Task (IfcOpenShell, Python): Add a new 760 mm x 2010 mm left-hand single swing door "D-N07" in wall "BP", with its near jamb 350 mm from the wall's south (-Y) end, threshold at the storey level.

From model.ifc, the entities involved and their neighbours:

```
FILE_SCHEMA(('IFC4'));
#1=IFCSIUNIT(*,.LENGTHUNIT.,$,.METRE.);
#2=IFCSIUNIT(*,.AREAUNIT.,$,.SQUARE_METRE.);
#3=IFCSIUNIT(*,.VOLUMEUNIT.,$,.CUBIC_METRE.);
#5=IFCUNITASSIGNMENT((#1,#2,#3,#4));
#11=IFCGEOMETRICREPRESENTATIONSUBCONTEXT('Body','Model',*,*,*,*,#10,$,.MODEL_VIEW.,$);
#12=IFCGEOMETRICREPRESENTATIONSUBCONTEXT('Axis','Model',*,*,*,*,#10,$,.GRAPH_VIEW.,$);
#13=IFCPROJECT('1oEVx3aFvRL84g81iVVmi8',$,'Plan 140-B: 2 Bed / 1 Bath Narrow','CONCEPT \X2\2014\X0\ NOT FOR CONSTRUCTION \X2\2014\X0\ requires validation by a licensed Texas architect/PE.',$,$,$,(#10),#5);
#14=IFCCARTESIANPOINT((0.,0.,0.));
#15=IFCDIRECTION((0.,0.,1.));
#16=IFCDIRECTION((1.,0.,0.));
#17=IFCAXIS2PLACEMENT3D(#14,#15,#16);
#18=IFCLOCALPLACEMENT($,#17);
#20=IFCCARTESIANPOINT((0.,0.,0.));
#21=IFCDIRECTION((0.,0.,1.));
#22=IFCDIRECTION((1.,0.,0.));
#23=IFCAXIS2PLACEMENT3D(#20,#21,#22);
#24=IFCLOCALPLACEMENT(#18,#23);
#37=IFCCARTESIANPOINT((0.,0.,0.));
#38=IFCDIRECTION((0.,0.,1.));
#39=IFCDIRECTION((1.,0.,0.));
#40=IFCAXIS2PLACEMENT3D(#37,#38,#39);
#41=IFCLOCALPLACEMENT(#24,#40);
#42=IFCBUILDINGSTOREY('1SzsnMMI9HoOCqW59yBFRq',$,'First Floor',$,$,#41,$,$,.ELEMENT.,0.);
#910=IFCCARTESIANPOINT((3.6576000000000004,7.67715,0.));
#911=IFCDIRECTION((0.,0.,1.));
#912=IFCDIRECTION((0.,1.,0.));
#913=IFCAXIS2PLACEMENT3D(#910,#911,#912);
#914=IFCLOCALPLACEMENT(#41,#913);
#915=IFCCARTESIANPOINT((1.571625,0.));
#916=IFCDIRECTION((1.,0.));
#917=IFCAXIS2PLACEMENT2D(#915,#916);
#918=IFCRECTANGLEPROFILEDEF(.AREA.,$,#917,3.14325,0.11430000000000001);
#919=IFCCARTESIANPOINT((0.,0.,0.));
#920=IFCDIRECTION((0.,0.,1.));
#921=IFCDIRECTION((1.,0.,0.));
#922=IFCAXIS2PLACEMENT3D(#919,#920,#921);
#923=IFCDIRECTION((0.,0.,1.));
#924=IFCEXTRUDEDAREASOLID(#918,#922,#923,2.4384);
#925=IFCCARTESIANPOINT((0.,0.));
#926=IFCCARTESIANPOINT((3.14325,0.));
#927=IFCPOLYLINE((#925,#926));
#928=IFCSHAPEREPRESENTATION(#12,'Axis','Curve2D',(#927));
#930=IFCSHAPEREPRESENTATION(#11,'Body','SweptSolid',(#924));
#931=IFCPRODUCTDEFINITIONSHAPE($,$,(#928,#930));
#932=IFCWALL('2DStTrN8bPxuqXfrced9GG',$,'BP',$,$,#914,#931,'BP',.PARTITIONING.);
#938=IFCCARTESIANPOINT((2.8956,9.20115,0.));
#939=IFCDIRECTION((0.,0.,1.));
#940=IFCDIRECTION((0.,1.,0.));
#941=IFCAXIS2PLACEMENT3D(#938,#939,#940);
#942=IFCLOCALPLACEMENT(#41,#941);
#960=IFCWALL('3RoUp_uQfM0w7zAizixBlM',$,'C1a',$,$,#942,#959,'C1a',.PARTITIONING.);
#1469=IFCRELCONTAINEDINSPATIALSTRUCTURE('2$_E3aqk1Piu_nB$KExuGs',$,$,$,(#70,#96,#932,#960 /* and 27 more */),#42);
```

```python
import numpy as np
import ifcopenshell
import ifcopenshell.api.feature
import ifcopenshell.api.geometry
import ifcopenshell.api.root
import ifcopenshell.api.spatial
import ifcopenshell.geom
import ifcopenshell.util.element
import ifcopenshell.util.placement
import ifcopenshell.util.representation
import ifcopenshell.util.shape
import ifcopenshell.util.unit

model = ifcopenshell.open("model.ifc")
unit_scale = ifcopenshell.util.unit.calculate_unit_scale(model)
settings = ifcopenshell.geom.settings()


def volume(element):
    """Net volume in cubic metres, openings subtracted."""
    shape = ifcopenshell.geom.create_shape(settings, element)
    return ifcopenshell.util.shape.get_volume(shape.geometry)


wall = model.by_guid("2DStTrN8bPxuqXfrced9GG")
storey = ifcopenshell.util.element.get_container(wall, ifc_class="IfcBuildingStorey")
context = ifcopenshell.util.representation.get_context(model, "Model", "Body", "MODEL_VIEW")
before = volume(wall)

width, height, from_end, sill = 0.76, 2.01, 0.35, 0.0  # metres

# The wall runs along its own X axis, and the end named is its -X end.
wall_shape = ifcopenshell.geom.create_shape(settings, wall)
x, y, z = ifcopenshell.util.shape.get_vertices(wall_shape.geometry).T
start = x.min() + from_end
face, thickness = float(y.min()), float(y.max() - y.min())
wall_matrix = ifcopenshell.util.placement.get_local_placement(wall.ObjectPlacement)
level = ifcopenshell.util.placement.get_local_placement(storey.ObjectPlacement)[2, 3]


def in_wall(x, y):
    """Placement at x, y metres in the wall's axes, at sill height."""
    matrix = wall_matrix.copy()
    matrix[:, 3] = wall_matrix @ np.array([x / unit_scale, y / unit_scale, 0.0, 1.0])
    matrix[2, 3] = level + sill / unit_scale
    return matrix


# Opening: a box that overshoots both wall faces by 50 mm.
opening = ifcopenshell.api.root.create_entity(model, ifc_class="IfcOpeningElement", predefined_type="OPENING")
box = ifcopenshell.api.geometry.add_wall_representation(
    model, context=context, length=width, height=height, thickness=thickness + 0.1
)
ifcopenshell.api.geometry.assign_representation(model, product=opening, representation=box)
ifcopenshell.api.geometry.edit_object_placement(model, product=opening, matrix=in_wall(start, face - 0.05), is_si=False)
ifcopenshell.api.feature.add_feature(model, feature=opening, element=wall)

door = ifcopenshell.api.root.create_entity(model, ifc_class="IfcDoor", name="D-N07", predefined_type="DOOR")
door.OverallWidth, door.OverallHeight = width / unit_scale, height / unit_scale
door.OperationType = "SINGLE_SWING_LEFT"
body = ifcopenshell.api.geometry.add_door_representation(
    model,
    context=context,
    overall_width=door.OverallWidth,
    overall_height=door.OverallHeight,
    operation_type="SINGLE_SWING_LEFT",
    lining_properties={"LiningDepth": thickness / unit_scale, "ThresholdDepth": thickness / unit_scale},
)
ifcopenshell.api.geometry.assign_representation(model, product=door, representation=body)
ifcopenshell.api.spatial.assign_container(model, products=[door], relating_structure=storey)
ifcopenshell.api.feature.add_filling(model, opening=opening, element=door)

# The lining spans the wall, so the door starts at the wall face.
ifcopenshell.api.geometry.edit_object_placement(model, product=door, matrix=in_wall(start, face), is_si=False)

after = volume(wall)

print(f"wall volume {before:.3f} -> {after:.3f} m3")

model.write("model_v2.ifc")
```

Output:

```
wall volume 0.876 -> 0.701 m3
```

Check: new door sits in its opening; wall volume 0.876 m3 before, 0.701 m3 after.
